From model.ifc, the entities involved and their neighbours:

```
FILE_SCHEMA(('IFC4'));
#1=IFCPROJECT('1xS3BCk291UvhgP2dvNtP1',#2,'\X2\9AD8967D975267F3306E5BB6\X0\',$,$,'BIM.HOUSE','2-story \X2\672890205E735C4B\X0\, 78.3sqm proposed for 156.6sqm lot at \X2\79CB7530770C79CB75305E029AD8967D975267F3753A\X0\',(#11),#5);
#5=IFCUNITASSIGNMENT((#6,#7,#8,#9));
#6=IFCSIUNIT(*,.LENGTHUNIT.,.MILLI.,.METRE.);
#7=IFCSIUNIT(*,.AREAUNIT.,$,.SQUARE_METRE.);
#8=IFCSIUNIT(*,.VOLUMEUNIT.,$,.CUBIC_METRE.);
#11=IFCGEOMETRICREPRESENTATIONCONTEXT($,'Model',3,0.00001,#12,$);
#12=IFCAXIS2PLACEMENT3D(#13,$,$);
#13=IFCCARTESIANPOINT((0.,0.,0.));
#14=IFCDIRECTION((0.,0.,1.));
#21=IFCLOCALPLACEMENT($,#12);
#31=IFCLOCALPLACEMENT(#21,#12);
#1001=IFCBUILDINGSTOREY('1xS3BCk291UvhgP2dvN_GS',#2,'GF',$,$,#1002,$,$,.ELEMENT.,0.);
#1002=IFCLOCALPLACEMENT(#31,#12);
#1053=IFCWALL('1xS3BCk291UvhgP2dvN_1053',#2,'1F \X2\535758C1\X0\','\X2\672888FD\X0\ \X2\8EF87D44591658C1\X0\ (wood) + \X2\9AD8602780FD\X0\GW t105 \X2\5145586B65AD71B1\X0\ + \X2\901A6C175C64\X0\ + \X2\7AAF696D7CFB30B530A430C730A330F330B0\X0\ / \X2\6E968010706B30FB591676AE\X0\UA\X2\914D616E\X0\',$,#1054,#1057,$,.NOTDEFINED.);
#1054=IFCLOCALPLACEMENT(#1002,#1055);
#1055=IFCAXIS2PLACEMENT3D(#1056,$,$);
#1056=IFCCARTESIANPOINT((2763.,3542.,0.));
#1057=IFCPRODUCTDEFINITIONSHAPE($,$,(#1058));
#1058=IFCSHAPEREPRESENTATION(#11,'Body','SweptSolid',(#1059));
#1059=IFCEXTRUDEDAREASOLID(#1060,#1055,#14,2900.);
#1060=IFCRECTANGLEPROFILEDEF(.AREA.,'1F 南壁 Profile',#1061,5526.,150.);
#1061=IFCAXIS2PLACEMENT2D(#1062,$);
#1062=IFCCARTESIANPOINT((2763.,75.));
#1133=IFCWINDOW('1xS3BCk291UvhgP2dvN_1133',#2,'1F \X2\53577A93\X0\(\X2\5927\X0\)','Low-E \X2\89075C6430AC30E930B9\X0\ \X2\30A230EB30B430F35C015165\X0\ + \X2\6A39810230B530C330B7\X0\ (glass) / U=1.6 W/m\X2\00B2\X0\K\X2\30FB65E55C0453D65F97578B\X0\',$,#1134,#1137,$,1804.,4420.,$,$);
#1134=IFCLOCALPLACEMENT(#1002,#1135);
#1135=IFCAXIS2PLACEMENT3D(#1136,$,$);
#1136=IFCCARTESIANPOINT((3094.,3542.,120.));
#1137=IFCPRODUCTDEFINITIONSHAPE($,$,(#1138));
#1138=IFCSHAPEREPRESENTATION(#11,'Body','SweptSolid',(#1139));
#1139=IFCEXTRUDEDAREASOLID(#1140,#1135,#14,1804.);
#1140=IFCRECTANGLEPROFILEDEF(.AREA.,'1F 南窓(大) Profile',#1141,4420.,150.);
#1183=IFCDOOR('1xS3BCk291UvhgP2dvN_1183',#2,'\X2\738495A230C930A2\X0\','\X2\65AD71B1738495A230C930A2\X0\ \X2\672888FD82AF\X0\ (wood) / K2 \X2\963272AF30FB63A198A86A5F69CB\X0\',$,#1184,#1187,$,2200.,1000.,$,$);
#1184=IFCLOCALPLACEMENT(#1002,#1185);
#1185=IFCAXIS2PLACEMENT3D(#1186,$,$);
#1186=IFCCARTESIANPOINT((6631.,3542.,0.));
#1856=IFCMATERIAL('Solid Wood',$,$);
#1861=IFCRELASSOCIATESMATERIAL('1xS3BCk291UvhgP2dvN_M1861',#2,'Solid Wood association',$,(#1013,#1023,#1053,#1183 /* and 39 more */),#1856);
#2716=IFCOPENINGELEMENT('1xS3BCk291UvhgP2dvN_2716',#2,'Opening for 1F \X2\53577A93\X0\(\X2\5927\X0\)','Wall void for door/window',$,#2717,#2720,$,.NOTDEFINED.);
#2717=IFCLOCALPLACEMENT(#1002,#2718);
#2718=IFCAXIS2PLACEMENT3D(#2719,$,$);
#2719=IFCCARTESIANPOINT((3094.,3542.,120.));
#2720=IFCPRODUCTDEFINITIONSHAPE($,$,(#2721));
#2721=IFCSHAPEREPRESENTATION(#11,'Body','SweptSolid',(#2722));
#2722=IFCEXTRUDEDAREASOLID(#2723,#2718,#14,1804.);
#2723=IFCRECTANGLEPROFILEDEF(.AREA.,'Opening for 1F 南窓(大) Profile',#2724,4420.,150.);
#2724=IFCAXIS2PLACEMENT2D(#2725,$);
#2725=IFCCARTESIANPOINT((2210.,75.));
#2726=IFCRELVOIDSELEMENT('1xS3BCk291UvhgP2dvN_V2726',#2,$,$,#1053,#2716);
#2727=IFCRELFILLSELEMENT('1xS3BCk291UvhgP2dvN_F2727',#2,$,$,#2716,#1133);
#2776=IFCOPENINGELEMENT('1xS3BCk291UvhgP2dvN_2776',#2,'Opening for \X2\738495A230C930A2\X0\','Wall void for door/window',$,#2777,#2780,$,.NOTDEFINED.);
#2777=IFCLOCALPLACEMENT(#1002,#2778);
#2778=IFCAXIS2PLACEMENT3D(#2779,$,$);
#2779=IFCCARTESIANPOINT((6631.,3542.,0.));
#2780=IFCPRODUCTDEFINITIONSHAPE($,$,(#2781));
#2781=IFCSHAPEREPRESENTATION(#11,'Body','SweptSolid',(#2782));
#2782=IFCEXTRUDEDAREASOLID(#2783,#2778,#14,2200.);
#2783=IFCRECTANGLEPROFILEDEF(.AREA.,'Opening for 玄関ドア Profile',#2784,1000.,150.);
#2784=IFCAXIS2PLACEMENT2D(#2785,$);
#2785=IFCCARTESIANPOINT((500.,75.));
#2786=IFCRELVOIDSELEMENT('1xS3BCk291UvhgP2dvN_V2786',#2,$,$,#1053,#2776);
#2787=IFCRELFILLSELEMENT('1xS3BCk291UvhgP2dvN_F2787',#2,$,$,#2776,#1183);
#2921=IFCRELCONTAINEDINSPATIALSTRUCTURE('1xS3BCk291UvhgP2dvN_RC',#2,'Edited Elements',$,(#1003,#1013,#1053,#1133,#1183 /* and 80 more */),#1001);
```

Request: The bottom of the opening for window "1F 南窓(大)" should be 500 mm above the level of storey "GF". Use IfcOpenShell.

```python
import numpy as np
import ifcopenshell
import ifcopenshell.api.geometry
import ifcopenshell.geom
import ifcopenshell.util.element
import ifcopenshell.util.placement
import ifcopenshell.util.shape
import ifcopenshell.util.unit

model = ifcopenshell.open("model.ifc")
unit_scale = ifcopenshell.util.unit.calculate_unit_scale(model)

window = model.by_guid("1xS3BCk291UvhgP2dvN_1133")
opening = window.FillsVoids[0].RelatingOpeningElement
storey = ifcopenshell.util.element.get_container(window, ifc_class="IfcBuildingStorey")
level = ifcopenshell.util.placement.get_local_placement(storey.ObjectPlacement)[2, 3]

# The opening's origin need not be at the sill, so measure its lowest point.
shape = ifcopenshell.geom.create_shape(ifcopenshell.geom.settings(), opening)
bottom = ifcopenshell.util.shape.get_shape_bottom_elevation(shape, shape.geometry) / unit_scale
dz = level + 0.5 / unit_scale - bottom

shift = np.array([0.0, 0.0, dz])
# The window is not placed relative to its opening, so move both.
for product in (opening, window):
    matrix = ifcopenshell.util.placement.get_local_placement(product.ObjectPlacement)
    matrix[:3, 3] += shift
    ifcopenshell.api.geometry.edit_object_placement(model, product=product, matrix=matrix, is_si=False)

print(f"moved by {dz * unit_scale:+.3f} m")

model.write("model_v2.ifc")
```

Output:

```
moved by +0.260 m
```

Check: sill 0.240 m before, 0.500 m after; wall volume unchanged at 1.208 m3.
